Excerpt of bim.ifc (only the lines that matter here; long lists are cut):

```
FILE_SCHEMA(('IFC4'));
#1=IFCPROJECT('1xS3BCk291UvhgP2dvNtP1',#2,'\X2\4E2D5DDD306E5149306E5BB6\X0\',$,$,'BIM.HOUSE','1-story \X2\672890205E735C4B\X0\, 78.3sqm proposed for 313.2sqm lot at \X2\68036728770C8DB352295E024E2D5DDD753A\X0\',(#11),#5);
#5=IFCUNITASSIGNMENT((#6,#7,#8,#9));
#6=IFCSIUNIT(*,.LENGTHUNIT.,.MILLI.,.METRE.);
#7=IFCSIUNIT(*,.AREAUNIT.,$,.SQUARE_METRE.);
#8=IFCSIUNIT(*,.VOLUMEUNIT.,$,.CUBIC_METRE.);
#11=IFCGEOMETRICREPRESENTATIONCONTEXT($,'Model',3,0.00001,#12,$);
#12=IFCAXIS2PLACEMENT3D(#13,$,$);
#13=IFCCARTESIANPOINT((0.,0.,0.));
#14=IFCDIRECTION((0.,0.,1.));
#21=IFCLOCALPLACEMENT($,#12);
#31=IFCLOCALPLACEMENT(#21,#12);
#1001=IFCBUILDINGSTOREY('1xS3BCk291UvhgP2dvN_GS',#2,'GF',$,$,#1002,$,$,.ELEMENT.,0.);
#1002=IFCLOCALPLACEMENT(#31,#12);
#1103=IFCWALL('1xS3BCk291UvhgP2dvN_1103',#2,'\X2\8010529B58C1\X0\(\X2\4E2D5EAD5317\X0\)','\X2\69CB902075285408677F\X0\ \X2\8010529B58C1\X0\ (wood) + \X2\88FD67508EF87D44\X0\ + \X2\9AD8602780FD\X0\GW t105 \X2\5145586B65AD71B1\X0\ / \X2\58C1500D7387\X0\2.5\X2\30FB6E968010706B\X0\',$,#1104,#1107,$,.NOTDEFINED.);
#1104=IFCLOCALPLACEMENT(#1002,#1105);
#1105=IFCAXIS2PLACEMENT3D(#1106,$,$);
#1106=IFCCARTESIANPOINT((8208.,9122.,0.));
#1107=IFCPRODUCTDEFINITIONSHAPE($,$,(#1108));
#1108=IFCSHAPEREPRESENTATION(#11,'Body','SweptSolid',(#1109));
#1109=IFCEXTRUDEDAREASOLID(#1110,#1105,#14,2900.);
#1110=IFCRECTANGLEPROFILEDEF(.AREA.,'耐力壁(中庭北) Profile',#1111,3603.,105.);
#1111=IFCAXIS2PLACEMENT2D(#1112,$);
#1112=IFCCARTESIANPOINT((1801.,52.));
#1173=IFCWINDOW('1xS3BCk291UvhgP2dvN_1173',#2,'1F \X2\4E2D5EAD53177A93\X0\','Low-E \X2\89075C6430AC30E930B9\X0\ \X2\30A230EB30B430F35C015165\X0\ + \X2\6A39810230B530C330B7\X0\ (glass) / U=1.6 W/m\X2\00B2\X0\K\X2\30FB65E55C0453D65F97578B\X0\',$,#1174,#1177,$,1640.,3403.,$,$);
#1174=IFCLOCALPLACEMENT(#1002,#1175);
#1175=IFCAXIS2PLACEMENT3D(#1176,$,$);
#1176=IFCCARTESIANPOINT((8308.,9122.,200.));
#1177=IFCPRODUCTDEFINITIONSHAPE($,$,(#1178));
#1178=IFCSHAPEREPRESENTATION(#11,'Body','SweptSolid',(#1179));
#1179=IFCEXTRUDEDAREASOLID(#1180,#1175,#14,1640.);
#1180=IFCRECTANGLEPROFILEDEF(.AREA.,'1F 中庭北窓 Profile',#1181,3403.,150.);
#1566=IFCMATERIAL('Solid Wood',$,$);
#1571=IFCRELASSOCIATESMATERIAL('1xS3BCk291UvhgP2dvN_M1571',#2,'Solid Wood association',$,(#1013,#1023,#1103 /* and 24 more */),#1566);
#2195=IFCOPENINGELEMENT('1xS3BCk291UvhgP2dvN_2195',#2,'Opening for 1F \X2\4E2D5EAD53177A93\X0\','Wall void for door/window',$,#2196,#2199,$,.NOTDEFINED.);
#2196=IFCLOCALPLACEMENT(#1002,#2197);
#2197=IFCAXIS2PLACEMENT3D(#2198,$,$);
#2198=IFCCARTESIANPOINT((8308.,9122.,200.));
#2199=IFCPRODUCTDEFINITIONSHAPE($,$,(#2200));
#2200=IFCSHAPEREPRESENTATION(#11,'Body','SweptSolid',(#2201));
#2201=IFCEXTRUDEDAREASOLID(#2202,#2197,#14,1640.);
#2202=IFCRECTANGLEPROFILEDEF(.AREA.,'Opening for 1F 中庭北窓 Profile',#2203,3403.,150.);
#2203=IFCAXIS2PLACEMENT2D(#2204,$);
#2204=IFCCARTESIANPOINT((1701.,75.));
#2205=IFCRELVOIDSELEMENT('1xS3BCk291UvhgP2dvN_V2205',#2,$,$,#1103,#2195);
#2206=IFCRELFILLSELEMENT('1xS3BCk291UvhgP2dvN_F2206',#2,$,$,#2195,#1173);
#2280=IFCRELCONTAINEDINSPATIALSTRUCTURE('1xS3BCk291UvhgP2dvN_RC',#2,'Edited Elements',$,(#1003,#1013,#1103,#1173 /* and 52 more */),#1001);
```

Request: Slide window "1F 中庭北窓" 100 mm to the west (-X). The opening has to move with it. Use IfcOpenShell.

```python
import ifcopenshell
import ifcopenshell.api.geometry
import ifcopenshell.util.placement
import ifcopenshell.util.unit

model = ifcopenshell.open("bim.ifc")
unit_scale = ifcopenshell.util.unit.calculate_unit_scale(model)

window = model.by_guid("1xS3BCk291UvhgP2dvN_1173")
opening = window.FillsVoids[0].RelatingOpeningElement
wall = opening.VoidsElements[0].RelatingBuildingElement

wall_matrix = ifcopenshell.util.placement.get_local_placement(wall.ObjectPlacement)
shift = wall_matrix[:3, 0] * -0.1 / unit_scale
before = ifcopenshell.util.placement.get_local_placement(window.ObjectPlacement)[:3, 3].copy()

# The window is not placed relative to its opening, so move both.
for product in (opening, window):
    matrix = ifcopenshell.util.placement.get_local_placement(product.ObjectPlacement)
    matrix[:3, 3] += shift
    ifcopenshell.api.geometry.edit_object_placement(model, product=product, matrix=matrix, is_si=False)

after = ifcopenshell.util.placement.get_local_placement(window.ObjectPlacement)[:3, 3]
print("window moved by", (after - before).round(3) + 0.0)

model.write("bim_edited.ifc")
```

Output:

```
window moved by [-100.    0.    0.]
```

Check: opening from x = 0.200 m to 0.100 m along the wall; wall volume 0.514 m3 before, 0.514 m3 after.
